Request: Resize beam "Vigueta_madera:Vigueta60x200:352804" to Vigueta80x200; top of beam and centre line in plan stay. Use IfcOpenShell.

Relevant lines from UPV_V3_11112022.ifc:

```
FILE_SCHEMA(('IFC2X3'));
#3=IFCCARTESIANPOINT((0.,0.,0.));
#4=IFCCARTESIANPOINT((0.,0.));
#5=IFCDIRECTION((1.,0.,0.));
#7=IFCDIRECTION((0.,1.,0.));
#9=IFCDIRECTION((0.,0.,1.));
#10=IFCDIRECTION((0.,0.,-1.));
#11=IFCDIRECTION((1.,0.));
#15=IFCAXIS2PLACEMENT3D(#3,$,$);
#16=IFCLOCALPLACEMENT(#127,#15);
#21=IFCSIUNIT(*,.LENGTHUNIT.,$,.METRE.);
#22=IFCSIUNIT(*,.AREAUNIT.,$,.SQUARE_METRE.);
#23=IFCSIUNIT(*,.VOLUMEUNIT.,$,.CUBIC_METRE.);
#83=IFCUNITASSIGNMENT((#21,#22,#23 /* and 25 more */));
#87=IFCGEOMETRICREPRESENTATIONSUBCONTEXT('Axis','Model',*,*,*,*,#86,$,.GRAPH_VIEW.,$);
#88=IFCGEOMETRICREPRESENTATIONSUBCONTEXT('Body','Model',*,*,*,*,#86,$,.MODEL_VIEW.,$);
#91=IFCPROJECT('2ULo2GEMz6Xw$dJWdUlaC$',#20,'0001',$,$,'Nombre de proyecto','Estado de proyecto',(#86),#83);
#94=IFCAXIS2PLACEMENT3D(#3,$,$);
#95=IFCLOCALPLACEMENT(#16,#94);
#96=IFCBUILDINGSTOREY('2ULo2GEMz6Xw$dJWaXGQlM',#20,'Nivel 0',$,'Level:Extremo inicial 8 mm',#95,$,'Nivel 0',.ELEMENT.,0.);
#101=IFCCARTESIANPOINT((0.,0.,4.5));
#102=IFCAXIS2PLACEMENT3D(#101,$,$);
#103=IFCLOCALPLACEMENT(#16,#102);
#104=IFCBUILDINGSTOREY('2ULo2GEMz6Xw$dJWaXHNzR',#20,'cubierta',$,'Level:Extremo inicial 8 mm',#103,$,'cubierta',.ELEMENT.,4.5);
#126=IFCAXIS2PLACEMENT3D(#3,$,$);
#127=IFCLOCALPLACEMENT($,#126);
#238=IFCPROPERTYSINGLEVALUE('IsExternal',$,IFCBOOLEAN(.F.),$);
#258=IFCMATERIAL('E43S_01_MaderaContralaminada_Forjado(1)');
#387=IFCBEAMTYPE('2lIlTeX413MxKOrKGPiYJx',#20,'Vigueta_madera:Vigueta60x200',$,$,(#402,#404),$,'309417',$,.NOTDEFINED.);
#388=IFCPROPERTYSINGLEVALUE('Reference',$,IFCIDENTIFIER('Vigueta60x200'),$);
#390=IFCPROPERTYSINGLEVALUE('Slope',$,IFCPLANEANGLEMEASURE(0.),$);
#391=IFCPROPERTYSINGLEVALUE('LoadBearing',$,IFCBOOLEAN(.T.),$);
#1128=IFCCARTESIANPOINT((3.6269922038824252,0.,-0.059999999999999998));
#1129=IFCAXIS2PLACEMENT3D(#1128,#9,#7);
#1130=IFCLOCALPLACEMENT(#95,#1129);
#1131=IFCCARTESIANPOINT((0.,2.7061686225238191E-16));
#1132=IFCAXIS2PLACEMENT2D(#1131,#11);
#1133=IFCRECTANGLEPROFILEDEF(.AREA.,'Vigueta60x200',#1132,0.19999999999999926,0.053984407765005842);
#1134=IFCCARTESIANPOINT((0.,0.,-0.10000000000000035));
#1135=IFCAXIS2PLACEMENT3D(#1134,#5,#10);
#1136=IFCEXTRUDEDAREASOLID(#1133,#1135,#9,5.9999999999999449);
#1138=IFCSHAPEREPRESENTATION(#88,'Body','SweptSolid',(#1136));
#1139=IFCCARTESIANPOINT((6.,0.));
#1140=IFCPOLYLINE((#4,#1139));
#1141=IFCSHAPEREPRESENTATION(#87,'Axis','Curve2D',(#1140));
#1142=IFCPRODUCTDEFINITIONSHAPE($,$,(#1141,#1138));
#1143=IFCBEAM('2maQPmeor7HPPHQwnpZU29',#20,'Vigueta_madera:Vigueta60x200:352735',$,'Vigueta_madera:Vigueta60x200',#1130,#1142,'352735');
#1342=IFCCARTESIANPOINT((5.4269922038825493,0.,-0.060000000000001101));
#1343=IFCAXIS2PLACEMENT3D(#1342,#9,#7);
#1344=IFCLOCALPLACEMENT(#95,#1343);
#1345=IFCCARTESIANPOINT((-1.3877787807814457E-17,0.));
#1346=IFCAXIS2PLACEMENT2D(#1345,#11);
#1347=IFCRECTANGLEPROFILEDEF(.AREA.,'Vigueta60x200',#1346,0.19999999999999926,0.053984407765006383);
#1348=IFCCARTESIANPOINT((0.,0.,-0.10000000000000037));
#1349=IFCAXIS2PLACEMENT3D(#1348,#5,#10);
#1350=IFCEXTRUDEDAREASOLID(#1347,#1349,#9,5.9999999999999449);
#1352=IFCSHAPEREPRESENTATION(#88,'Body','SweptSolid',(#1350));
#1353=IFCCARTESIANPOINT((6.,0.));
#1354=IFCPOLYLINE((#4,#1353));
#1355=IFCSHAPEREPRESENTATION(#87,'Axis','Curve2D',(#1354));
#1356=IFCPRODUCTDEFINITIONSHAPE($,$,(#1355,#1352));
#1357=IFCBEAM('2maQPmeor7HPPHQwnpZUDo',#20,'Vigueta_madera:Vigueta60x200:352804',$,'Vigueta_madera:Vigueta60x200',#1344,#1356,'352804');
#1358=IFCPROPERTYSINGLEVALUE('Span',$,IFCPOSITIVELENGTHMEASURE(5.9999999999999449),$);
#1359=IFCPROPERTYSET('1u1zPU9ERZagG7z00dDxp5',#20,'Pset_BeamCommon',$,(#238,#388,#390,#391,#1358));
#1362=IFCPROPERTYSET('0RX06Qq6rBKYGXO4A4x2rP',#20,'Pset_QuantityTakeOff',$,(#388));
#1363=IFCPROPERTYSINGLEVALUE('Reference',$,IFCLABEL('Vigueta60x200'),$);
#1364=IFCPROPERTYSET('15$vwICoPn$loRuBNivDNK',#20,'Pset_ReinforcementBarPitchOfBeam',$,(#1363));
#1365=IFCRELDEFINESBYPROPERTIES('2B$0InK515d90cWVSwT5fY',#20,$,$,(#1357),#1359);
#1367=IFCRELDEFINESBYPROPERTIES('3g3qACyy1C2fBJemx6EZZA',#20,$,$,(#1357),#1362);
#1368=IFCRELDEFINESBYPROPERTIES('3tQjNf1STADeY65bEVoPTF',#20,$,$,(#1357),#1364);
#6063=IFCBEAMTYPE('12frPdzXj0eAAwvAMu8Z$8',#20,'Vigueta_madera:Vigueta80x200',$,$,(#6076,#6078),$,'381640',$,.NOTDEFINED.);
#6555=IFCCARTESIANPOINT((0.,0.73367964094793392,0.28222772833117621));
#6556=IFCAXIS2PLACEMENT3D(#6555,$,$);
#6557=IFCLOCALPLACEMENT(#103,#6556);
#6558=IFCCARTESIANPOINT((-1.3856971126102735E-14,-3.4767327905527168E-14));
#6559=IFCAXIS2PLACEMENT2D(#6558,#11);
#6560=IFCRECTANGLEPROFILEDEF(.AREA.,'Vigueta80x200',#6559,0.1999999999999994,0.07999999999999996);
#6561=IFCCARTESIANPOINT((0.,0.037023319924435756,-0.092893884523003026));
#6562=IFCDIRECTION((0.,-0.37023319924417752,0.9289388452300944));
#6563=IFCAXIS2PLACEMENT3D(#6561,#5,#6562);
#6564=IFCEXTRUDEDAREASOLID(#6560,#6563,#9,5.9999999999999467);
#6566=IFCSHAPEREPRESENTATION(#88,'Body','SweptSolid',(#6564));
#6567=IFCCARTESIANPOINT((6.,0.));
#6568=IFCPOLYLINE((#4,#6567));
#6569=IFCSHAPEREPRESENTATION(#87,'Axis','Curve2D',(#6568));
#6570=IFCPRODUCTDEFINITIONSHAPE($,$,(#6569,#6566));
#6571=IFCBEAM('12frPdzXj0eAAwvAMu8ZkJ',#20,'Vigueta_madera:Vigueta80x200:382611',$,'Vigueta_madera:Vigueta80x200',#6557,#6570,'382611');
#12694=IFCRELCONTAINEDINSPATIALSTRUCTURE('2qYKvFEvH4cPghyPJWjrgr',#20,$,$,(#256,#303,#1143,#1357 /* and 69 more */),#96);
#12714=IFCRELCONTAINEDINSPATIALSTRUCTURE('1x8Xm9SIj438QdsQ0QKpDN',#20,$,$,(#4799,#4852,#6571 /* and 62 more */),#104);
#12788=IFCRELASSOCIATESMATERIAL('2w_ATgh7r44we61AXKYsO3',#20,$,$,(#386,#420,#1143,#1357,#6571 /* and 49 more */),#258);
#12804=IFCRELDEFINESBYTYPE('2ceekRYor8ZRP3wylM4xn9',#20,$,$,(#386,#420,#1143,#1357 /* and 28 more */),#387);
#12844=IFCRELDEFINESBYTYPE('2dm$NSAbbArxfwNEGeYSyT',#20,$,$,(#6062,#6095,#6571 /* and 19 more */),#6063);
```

```python
import ifcopenshell
import ifcopenshell.api.pset
import ifcopenshell.api.type
import ifcopenshell.util.element
import ifcopenshell.util.representation

model = ifcopenshell.open("UPV_V3_11112022.ifc")

member = model.by_guid("2maQPmeor7HPPHQwnpZUDo")
source = next(p for p in model.by_type("IfcRectangleProfileDef") if p.ProfileName == "Vigueta80x200")

body = ifcopenshell.util.representation.get_representation(member, "Model", "Body")
solid = body.Items[0]
old_profile = solid.SweptArea

# Copy the section's sizes but keep this member's own profile position.
profile = ifcopenshell.util.element.copy(model, source)
# Profiles are centred, so shift by half the change in depth to hold the top.
shift = (old_profile.XDim - profile.XDim) / 2
x, y = old_profile.Position.Location.Coordinates
up = (-1.0, 0.0)  # upwards, in the solid's own plane
location = model.createIfcCartesianPoint((x + up[0] * shift, y + up[1] * shift))
profile.Position = model.createIfcAxis2Placement2D(location, old_profile.Position.RefDirection)
solid.SweptArea = profile
if not model.get_total_inverses(old_profile):
    ifcopenshell.util.element.remove_deep2(model, old_profile)

new_type = model.by_guid("12frPdzXj0eAAwvAMu8Z$8")
ifcopenshell.api.type.assign_type(
    model, related_objects=[member], relating_type=new_type, should_map_representations=False
)
member.Name = member.Name.replace("Vigueta60x200", "Vigueta80x200")
member.ObjectType = "Vigueta_madera:Vigueta80x200"
pset = model.by_id(ifcopenshell.util.element.get_pset(member, "Pset_BeamCommon", should_inherit=False)["id"])
ifcopenshell.api.pset.edit_pset(model, pset=pset, properties={"Reference": "Vigueta80x200"})
pset = model.by_id(ifcopenshell.util.element.get_pset(member, "Pset_QuantityTakeOff", should_inherit=False)["id"])
ifcopenshell.api.pset.edit_pset(model, pset=pset, properties={"Reference": "Vigueta80x200"})
pset = model.by_id(ifcopenshell.util.element.get_pset(member, "Pset_ReinforcementBarPitchOfBeam", should_inherit=False)["id"])
ifcopenshell.api.pset.edit_pset(model, pset=pset, properties={"Reference": "Vigueta80x200"})

print(solid.SweptArea)

model.write("UPV_V3_11112022-out.ifc")
```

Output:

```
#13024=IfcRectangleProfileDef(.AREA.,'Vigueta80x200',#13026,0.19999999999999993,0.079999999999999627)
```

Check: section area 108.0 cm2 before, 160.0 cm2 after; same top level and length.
